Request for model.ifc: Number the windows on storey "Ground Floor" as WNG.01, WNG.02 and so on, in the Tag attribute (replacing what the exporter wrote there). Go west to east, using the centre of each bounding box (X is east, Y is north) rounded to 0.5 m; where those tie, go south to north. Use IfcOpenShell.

First a look at what the model holds.

```python
import ifcopenshell
import ifcopenshell.util.element
import ifcopenshell.util.placement

model = ifcopenshell.open("model.ifc")
print(model.schema)
storey = next(s for s in model.by_type("IfcBuildingStorey") if s.Name == "Ground Floor")
windows = [e for e in ifcopenshell.util.element.get_decomposition(storey) if e.is_a("IfcWindow")]
for e in sorted(windows, key=lambda e: e.id()):
    origin = ifcopenshell.util.placement.get_local_placement(e.ObjectPlacement)[:3, 3]
    print(e.id(), e.Tag, e.Name, origin.round(2) + 0.0, sep=" | ")
```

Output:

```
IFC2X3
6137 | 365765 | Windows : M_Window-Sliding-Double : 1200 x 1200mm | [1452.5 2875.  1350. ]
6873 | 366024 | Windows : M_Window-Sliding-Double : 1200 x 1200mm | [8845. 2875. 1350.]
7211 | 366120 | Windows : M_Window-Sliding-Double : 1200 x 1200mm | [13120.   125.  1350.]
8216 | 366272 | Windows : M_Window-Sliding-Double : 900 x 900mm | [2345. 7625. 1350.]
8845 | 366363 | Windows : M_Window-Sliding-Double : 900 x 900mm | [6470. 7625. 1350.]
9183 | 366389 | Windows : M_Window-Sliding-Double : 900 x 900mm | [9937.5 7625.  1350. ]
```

```python
import ifcopenshell
import ifcopenshell.geom
import ifcopenshell.util.element
import ifcopenshell.util.shape

model = ifcopenshell.open("model.ifc")
settings = ifcopenshell.geom.settings()
settings.set("use-world-coords", True)


def centre(element):
    shape = ifcopenshell.geom.create_shape(settings, element)
    return ifcopenshell.util.shape.get_bbox_centroid(shape.geometry)


storey = next(s for s in model.by_type("IfcBuildingStorey") if s.Name == "Ground Floor")
windows = [e for e in ifcopenshell.util.element.get_decomposition(storey) if e.is_a("IfcWindow")]

# Insertion points can sit at a corner or the storey origin, so sort by the geometry (in metres).
centres = {e: centre(e) for e in windows}
windows.sort(key=lambda e: (round(centres[e][0] / 0.5), centres[e][1]))

for i, e in enumerate(windows, start=1):
    number = f"WNG.{i:02d}"
    e.Tag = number
    print(e.id(), number)

model.write("model-out.ifc")
```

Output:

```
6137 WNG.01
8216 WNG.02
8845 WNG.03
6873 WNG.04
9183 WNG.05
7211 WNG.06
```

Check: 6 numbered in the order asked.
